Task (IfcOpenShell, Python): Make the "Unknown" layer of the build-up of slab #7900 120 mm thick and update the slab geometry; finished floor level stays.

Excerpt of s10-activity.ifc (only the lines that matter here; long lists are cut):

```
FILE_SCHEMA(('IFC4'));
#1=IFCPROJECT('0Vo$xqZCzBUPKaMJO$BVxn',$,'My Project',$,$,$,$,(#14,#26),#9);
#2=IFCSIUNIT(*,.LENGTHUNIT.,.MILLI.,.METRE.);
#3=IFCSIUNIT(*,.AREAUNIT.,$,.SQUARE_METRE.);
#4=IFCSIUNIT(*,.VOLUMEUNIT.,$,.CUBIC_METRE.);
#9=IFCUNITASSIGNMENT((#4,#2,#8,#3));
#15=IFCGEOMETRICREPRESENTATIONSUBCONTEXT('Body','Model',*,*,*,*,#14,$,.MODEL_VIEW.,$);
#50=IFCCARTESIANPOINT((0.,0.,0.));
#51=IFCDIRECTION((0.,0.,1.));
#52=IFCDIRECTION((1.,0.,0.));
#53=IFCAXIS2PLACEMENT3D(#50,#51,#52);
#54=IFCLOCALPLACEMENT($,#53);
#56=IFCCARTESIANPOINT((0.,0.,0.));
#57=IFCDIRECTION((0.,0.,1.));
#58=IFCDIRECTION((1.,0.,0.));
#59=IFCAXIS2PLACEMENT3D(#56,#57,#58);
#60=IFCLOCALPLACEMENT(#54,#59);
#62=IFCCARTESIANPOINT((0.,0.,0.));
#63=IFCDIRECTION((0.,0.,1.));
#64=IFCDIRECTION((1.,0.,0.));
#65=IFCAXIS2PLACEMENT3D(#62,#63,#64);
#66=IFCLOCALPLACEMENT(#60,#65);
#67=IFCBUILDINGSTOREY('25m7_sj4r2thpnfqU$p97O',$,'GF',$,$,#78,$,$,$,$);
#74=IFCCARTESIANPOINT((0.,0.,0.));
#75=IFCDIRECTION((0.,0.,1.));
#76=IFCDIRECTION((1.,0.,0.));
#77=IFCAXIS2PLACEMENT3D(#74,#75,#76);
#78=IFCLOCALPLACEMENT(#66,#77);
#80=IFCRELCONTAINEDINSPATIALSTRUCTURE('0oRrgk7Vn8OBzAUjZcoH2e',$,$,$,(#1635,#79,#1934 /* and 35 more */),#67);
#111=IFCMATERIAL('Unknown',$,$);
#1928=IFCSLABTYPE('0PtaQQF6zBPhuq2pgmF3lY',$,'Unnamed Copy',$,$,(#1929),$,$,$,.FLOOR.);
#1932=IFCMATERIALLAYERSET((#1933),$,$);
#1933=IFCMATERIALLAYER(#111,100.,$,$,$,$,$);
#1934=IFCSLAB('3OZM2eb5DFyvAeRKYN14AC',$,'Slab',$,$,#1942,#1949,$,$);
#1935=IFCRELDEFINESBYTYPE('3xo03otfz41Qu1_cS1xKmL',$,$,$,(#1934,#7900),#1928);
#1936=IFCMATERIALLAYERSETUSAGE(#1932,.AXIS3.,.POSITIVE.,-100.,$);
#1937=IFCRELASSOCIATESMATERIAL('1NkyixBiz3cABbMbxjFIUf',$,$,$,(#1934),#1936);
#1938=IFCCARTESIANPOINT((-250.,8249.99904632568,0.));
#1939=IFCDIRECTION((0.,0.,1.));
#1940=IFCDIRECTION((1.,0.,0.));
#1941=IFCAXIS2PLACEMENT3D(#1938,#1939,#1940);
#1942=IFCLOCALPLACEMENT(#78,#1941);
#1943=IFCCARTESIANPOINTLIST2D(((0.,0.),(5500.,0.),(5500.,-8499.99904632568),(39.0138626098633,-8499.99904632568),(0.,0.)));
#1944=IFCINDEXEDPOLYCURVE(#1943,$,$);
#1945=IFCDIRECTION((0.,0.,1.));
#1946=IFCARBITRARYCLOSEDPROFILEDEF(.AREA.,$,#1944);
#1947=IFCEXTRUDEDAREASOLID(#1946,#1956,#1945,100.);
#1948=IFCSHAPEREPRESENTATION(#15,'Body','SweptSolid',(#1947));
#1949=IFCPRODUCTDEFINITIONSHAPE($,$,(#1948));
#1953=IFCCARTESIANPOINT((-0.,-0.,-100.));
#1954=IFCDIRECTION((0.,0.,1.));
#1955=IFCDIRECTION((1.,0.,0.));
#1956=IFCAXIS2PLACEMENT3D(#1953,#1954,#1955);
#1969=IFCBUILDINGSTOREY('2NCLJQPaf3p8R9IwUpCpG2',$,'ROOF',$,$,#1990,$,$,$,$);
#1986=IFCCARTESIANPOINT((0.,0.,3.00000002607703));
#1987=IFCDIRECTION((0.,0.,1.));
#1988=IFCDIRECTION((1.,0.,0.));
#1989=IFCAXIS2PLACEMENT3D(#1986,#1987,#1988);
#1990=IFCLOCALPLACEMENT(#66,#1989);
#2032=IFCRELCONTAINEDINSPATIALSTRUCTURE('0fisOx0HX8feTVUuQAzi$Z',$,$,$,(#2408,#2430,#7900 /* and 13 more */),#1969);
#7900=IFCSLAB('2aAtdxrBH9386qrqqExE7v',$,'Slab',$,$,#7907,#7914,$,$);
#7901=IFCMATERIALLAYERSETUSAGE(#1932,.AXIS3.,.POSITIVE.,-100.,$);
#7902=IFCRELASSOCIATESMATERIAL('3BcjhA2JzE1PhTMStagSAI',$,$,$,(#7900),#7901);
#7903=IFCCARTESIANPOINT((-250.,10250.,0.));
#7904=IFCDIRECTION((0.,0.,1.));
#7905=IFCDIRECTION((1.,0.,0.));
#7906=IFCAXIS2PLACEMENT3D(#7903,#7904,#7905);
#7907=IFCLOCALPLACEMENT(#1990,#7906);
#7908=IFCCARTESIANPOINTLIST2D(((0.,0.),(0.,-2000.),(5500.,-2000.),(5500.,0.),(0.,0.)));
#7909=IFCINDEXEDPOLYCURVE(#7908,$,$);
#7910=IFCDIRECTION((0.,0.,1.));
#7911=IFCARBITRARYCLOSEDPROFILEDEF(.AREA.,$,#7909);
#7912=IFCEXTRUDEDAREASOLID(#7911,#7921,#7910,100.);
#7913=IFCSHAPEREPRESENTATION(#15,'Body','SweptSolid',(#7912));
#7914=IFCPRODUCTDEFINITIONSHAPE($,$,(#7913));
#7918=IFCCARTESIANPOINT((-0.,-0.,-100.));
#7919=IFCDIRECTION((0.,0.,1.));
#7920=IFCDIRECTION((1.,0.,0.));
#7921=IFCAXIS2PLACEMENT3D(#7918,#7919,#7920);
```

```python
import ifcopenshell
import ifcopenshell.util.element
import ifcopenshell.util.representation
import ifcopenshell.util.unit

model = ifcopenshell.open("s10-activity.ifc")
unit_scale = ifcopenshell.util.unit.calculate_unit_scale(model)

layer_set = model.by_id(1932)
layer = next(l for l in layer_set.MaterialLayers if l.Material and l.Material.Name == "Unknown")
change = 0.12 / unit_scale - layer.LayerThickness
layer.LayerThickness += change

# The layer set is shared, so every slab that uses it gets the new thickness.
slabs = [e for e in ifcopenshell.util.element.get_elements_by_material(model, layer_set) if e.is_a("IfcSlab")]
for slab in sorted(slabs, key=lambda e: e.id()):
    body = ifcopenshell.util.representation.get_representation(slab, "Model", "Body")
    solid = body.Items[0]
    old_depth = solid.Depth
    solid.Depth += change
    # Extruded upwards: lower the start of the extrusion so the top stays.
    x, y, z = solid.Position.Location.Coordinates
    solid.Position.Location = model.createIfcCartesianPoint((x, y, z - change))
    print(slab.id(), f"{old_depth:g} -> {solid.Depth:g}")

# The layers are counted up from the underside, which has moved.
for usage in {ifcopenshell.util.element.get_material(slab) for slab in slabs}:
    usage.OffsetFromReferenceLine -= change

model.write("s10-activity-out.ifc")
```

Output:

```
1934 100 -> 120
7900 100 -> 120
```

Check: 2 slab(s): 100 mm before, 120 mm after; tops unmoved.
